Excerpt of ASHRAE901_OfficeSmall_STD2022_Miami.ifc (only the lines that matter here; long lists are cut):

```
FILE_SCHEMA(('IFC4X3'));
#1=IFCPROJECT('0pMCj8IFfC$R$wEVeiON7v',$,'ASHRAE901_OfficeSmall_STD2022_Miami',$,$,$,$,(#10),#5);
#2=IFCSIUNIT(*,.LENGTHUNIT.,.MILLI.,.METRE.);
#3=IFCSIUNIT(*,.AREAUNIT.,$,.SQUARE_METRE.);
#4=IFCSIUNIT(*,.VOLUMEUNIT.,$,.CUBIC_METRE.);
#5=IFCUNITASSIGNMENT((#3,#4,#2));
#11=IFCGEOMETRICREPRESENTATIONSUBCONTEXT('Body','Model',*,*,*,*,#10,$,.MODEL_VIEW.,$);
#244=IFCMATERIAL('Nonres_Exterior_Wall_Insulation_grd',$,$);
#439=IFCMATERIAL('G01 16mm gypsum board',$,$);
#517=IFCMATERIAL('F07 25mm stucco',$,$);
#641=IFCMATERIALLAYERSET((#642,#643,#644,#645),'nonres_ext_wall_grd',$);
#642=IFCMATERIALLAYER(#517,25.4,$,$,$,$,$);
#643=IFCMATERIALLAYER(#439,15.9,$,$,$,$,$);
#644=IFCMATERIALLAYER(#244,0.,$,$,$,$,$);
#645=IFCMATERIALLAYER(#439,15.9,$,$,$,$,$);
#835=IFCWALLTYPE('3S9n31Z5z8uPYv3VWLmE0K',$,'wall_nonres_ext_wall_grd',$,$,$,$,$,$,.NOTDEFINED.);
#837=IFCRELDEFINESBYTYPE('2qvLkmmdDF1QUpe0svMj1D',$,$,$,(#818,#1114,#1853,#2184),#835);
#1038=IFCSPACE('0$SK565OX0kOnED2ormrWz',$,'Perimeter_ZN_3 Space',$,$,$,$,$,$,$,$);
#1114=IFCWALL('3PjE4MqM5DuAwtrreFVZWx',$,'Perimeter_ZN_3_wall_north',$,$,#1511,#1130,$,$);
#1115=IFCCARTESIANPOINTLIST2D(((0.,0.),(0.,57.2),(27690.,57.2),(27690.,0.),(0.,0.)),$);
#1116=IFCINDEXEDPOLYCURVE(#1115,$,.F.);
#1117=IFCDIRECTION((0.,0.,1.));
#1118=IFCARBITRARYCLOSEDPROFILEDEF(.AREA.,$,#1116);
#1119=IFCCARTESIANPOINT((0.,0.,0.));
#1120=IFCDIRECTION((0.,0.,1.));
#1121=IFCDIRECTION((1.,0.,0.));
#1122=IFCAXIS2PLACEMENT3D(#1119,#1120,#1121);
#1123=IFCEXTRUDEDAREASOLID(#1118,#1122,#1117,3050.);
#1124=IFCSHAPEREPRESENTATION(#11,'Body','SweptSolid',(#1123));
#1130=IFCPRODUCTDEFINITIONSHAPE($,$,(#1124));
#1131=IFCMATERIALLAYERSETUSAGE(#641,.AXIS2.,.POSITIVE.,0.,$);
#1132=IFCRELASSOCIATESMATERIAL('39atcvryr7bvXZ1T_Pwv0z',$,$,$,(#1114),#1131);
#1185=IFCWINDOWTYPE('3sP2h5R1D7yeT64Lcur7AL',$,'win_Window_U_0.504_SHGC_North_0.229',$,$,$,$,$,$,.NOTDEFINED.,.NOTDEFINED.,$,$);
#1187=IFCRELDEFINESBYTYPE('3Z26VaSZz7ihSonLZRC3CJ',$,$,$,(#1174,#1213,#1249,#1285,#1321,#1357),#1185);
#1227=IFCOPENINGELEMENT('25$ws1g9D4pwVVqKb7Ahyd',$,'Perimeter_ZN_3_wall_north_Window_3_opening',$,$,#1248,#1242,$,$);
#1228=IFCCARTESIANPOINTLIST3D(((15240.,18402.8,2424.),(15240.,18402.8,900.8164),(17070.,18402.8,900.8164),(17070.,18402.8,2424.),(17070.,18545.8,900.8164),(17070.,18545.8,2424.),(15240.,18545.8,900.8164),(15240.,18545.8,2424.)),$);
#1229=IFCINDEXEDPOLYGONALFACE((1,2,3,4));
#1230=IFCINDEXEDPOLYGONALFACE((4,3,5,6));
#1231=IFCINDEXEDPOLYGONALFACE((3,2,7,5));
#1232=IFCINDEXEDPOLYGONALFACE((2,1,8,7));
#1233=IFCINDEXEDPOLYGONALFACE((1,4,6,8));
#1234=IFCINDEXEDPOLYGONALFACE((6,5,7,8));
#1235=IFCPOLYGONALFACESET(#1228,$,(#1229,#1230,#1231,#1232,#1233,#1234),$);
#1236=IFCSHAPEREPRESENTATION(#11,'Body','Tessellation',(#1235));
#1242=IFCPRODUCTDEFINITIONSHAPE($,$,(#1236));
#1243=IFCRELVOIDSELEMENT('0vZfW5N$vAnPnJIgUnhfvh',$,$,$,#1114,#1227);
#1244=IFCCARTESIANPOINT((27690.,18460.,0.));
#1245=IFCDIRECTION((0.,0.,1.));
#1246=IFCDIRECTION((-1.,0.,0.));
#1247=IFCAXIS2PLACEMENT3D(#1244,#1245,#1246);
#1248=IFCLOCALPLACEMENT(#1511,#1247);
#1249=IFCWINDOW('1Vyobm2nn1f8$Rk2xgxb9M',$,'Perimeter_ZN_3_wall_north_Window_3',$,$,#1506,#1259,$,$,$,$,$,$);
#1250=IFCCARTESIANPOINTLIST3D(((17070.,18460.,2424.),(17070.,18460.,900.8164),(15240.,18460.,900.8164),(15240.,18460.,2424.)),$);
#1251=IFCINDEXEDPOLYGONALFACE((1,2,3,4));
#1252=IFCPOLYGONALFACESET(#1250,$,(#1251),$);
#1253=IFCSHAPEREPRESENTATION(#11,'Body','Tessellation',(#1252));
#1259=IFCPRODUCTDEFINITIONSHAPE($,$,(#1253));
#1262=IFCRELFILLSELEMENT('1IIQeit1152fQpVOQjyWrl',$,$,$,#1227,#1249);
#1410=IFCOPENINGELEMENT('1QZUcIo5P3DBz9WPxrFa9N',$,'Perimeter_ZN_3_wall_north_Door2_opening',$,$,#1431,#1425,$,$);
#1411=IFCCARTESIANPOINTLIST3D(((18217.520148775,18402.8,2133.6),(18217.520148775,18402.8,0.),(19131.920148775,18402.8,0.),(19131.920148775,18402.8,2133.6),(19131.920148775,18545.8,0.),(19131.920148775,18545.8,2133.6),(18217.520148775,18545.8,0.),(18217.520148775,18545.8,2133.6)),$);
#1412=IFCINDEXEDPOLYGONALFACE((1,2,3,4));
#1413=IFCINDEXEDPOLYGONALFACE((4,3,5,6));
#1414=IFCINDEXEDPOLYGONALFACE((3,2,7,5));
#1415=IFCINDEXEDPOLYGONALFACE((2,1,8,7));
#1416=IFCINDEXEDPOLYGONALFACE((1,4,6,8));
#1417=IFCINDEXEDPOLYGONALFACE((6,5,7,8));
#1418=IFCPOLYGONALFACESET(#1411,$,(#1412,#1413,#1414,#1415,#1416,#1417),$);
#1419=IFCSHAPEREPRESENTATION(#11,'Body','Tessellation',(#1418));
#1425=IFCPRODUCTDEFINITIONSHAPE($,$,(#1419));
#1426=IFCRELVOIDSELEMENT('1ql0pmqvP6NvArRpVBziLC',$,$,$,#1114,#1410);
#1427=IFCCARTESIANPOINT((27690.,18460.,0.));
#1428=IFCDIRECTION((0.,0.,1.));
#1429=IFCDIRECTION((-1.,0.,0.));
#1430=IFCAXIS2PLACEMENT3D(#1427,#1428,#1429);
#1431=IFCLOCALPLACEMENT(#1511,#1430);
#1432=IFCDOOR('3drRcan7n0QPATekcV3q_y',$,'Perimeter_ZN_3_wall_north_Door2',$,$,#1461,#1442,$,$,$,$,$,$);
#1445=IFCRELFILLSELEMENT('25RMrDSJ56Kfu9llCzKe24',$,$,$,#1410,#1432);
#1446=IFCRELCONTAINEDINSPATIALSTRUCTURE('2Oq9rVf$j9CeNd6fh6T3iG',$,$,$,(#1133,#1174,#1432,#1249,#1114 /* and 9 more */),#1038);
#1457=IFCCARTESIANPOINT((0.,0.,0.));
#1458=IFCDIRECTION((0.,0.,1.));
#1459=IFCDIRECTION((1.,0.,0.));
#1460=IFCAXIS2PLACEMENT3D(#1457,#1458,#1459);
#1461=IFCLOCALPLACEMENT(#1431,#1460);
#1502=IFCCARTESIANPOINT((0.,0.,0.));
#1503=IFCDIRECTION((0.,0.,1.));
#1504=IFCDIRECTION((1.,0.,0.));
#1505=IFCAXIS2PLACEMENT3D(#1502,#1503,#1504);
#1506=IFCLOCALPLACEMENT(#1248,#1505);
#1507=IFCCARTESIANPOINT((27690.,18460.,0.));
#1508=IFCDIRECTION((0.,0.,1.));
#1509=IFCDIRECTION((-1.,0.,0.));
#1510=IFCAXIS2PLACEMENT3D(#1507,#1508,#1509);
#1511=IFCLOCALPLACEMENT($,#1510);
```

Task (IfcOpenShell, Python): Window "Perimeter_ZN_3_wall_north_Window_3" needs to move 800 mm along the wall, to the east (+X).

```python
import ifcopenshell
import ifcopenshell.api.geometry
import ifcopenshell.util.placement

model = ifcopenshell.open("ASHRAE901_OfficeSmall_STD2022_Miami.ifc")

window = model.by_id(1249)
opening = window.FillsVoids[0].RelatingOpeningElement
wall = opening.VoidsElements[0].RelatingBuildingElement

wall_matrix = ifcopenshell.util.placement.get_local_placement(wall.ObjectPlacement)
shift = wall_matrix[:3, 0] * -800.0
before = ifcopenshell.util.placement.get_local_placement(window.ObjectPlacement)[:3, 3].copy()

# The window is placed relative to its opening, so it follows when the opening moves.
matrix = ifcopenshell.util.placement.get_local_placement(opening.ObjectPlacement)
matrix[:3, 3] += shift
ifcopenshell.api.geometry.edit_object_placement(
    model, product=opening, matrix=matrix, is_si=False, should_transform_children=True
)

after = ifcopenshell.util.placement.get_local_placement(window.ObjectPlacement)[:3, 3]
print("window moved by", (after - before).round(3) + 0.0)

model.write("ASHRAE901_OfficeSmall_STD2022_Miami_rev.ifc")
```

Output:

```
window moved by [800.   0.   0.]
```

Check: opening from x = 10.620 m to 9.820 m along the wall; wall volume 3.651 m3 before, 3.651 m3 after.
